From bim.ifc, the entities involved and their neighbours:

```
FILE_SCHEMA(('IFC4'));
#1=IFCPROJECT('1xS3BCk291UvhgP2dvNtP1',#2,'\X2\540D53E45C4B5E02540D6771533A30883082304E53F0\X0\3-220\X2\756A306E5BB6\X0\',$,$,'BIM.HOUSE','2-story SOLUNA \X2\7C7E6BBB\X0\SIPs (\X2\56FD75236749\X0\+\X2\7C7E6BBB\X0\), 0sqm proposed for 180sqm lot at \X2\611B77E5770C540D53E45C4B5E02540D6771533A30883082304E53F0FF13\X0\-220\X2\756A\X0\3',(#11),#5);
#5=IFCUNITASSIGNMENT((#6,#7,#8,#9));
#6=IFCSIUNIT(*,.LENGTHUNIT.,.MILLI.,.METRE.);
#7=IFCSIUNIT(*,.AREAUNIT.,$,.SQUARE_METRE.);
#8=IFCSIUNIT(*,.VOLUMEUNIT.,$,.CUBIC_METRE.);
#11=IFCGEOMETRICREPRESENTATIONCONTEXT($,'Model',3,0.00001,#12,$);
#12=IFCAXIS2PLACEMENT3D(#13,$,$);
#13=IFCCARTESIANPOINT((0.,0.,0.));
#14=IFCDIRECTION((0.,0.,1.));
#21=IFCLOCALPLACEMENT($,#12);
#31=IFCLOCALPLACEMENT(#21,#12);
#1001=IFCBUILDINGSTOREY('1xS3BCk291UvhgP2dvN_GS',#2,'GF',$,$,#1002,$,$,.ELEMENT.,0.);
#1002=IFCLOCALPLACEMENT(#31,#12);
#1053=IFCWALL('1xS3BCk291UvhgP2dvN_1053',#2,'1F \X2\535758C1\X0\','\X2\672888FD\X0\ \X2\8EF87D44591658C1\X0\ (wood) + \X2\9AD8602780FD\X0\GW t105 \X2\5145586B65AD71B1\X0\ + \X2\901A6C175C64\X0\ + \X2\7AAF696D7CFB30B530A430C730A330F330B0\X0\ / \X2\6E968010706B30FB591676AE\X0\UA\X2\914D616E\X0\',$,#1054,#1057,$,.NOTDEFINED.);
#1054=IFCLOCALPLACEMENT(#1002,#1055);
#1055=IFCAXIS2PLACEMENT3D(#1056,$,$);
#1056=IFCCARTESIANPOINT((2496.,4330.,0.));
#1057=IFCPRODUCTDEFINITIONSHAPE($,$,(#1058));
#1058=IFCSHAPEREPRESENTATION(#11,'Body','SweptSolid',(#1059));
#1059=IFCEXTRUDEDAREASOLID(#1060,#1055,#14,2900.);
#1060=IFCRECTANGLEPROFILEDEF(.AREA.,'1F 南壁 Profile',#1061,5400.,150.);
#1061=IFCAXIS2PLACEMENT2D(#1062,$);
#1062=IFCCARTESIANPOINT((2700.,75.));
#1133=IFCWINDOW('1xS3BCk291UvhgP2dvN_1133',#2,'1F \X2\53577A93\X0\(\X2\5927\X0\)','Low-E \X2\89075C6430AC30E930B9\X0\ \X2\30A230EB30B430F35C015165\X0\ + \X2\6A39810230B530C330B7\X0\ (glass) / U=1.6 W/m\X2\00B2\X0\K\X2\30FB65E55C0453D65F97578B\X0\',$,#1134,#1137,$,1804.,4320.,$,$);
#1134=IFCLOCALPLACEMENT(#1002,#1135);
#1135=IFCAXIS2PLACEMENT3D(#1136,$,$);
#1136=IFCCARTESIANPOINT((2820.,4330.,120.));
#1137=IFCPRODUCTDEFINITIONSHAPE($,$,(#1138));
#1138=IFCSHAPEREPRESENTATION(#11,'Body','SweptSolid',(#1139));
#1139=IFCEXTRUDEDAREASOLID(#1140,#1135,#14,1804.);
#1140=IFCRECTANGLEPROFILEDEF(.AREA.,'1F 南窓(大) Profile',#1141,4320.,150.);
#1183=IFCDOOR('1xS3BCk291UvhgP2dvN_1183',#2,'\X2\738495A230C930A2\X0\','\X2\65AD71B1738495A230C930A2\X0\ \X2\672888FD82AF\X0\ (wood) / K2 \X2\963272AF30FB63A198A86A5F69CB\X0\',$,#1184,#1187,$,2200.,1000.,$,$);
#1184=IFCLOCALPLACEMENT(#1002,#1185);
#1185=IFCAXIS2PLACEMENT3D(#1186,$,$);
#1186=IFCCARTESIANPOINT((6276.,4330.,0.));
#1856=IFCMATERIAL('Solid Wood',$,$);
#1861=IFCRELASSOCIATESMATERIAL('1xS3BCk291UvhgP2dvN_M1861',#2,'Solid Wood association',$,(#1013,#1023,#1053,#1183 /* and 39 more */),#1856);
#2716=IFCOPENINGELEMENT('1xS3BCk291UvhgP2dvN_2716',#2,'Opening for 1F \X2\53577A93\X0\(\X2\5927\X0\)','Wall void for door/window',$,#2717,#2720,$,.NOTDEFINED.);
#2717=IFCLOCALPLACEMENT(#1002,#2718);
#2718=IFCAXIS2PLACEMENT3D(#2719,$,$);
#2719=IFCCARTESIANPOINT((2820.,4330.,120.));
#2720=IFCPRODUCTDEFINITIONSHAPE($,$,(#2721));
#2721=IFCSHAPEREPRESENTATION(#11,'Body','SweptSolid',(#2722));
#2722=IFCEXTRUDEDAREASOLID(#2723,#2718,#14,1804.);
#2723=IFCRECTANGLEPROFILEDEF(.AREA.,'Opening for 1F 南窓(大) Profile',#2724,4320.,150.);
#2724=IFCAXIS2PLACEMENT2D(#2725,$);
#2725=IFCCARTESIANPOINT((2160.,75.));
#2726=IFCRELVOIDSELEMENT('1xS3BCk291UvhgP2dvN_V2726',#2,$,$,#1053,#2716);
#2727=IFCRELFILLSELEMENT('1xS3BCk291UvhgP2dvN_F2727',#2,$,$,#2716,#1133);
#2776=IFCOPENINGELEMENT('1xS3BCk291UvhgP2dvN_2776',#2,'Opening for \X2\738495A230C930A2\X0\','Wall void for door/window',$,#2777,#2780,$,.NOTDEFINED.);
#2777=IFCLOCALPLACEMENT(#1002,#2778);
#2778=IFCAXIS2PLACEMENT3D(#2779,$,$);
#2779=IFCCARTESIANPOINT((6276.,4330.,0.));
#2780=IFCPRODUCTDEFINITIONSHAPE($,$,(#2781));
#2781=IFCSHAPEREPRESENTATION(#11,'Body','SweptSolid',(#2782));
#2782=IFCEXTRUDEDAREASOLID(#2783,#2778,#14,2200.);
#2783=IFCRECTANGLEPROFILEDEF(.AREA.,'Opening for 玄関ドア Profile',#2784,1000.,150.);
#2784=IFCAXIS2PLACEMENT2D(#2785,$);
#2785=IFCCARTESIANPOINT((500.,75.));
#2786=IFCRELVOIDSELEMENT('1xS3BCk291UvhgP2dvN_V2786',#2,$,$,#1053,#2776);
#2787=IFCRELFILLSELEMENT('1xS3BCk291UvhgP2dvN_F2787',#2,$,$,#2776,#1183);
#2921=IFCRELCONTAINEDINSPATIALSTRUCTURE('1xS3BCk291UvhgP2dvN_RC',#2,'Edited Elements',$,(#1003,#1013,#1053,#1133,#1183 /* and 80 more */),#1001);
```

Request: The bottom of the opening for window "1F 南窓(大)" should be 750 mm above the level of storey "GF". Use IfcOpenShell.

```python
import numpy as np
import ifcopenshell
import ifcopenshell.api.geometry
import ifcopenshell.geom
import ifcopenshell.util.element
import ifcopenshell.util.placement
import ifcopenshell.util.shape
import ifcopenshell.util.unit

model = ifcopenshell.open("bim.ifc")
unit_scale = ifcopenshell.util.unit.calculate_unit_scale(model)

window = model.by_guid("1xS3BCk291UvhgP2dvN_1133")
opening = window.FillsVoids[0].RelatingOpeningElement
storey = ifcopenshell.util.element.get_container(window, ifc_class="IfcBuildingStorey")
level = ifcopenshell.util.placement.get_local_placement(storey.ObjectPlacement)[2, 3]

# The opening's origin need not be at the sill, so measure its lowest point.
shape = ifcopenshell.geom.create_shape(ifcopenshell.geom.settings(), opening)
bottom = ifcopenshell.util.shape.get_shape_bottom_elevation(shape, shape.geometry) / unit_scale
dz = level + 0.75 / unit_scale - bottom

shift = np.array([0.0, 0.0, dz])
# The window is not placed relative to its opening, so move both.
for product in (opening, window):
    matrix = ifcopenshell.util.placement.get_local_placement(product.ObjectPlacement)
    matrix[:3, 3] += shift
    ifcopenshell.api.geometry.edit_object_placement(model, product=product, matrix=matrix, is_si=False)

print(f"moved by {dz * unit_scale:+.3f} m")

model.write("bim_v2.ifc")
```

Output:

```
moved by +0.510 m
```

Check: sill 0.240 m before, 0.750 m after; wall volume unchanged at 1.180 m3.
